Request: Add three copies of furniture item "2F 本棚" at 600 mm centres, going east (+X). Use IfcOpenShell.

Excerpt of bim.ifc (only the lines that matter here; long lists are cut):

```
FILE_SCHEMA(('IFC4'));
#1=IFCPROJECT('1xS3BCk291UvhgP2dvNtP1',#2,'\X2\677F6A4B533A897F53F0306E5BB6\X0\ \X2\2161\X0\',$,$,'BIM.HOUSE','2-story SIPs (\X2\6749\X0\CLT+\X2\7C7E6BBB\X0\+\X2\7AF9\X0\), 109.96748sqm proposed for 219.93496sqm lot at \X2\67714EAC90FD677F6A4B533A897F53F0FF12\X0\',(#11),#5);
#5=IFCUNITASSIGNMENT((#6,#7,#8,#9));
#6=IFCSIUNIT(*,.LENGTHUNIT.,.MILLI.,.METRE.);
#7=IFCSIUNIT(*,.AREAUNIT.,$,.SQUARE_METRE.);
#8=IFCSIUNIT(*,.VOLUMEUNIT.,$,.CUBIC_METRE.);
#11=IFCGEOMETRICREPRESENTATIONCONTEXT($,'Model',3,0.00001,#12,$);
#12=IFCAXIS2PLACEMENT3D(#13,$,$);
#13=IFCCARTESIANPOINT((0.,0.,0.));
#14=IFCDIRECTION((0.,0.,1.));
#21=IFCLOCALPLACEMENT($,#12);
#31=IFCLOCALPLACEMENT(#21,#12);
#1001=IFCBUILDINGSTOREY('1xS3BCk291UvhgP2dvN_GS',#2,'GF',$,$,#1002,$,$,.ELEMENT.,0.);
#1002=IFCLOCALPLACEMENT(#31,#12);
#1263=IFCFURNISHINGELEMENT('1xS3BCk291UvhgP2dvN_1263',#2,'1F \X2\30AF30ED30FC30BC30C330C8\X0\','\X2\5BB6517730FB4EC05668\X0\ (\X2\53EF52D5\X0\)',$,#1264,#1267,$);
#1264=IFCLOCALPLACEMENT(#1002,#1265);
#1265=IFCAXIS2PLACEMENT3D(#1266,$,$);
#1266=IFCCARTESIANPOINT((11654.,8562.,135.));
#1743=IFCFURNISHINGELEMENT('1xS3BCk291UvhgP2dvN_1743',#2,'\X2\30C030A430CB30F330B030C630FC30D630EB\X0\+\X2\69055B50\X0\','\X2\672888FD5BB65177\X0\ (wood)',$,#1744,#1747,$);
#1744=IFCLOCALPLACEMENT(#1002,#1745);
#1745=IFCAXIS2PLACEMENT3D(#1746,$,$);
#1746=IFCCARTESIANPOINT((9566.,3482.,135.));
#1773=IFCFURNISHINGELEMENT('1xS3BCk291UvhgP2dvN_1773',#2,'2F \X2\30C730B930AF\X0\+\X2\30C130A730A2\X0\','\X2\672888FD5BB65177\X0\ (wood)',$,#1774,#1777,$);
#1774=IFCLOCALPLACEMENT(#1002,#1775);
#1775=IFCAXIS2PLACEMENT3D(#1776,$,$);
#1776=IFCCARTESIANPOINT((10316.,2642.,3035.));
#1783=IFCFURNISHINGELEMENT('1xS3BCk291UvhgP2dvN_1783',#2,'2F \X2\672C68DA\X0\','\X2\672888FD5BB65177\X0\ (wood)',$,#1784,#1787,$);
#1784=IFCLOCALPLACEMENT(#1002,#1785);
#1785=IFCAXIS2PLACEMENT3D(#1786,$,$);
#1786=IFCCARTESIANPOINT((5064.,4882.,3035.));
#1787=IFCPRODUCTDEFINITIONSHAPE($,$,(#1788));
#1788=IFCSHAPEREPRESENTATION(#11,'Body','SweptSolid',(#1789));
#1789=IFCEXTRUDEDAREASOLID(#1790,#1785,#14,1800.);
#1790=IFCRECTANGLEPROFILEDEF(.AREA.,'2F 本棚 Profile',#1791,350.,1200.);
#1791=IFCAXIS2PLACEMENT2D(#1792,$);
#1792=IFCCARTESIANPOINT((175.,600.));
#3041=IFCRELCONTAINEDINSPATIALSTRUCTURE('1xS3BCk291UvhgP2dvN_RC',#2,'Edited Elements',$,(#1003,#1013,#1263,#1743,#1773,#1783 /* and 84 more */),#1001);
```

```python
import numpy as np
import ifcopenshell
import ifcopenshell.api.geometry
import ifcopenshell.api.root
import ifcopenshell.util.element
import ifcopenshell.util.placement
import ifcopenshell.util.unit

model = ifcopenshell.open("bim.ifc")
unit_scale = ifcopenshell.util.unit.calculate_unit_scale(model)


def reuse_history(source, copy):
    """copy_class also copies each property set's owner history, people and application; keep the originals."""
    for rel in copy.IsDefinedBy:
        if rel.is_a("IfcRelDefinesByProperties") and (history := rel.RelatingPropertyDefinition.OwnerHistory):
            rel.RelatingPropertyDefinition.OwnerHistory = source.OwnerHistory
            ifcopenshell.util.element.remove_deep2(model, history)


source = model.by_id(1783)
base = ifcopenshell.util.placement.get_local_placement(source.ObjectPlacement)
step = np.array([1.0, 0.0, 0.0]) * 0.6 / unit_scale

for i in range(1, 4):
    copy = ifcopenshell.api.root.copy_class(model, product=source)
    copy.Representation = ifcopenshell.util.element.copy_deep(
        model, source.Representation, exclude=["IfcGeometricRepresentationContext", "IfcRepresentationMap"]
    )
    reuse_history(source, copy)
    matrix = base.copy()
    matrix[:3, 3] += i * step
    print("added at", matrix[:3, 3].round(3) + 0.0)
    ifcopenshell.api.geometry.edit_object_placement(model, product=copy, matrix=matrix, is_si=False)

model.write("bim_v2.ifc")
```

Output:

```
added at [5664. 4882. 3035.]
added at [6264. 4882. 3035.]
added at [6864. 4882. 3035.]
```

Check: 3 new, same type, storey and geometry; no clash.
